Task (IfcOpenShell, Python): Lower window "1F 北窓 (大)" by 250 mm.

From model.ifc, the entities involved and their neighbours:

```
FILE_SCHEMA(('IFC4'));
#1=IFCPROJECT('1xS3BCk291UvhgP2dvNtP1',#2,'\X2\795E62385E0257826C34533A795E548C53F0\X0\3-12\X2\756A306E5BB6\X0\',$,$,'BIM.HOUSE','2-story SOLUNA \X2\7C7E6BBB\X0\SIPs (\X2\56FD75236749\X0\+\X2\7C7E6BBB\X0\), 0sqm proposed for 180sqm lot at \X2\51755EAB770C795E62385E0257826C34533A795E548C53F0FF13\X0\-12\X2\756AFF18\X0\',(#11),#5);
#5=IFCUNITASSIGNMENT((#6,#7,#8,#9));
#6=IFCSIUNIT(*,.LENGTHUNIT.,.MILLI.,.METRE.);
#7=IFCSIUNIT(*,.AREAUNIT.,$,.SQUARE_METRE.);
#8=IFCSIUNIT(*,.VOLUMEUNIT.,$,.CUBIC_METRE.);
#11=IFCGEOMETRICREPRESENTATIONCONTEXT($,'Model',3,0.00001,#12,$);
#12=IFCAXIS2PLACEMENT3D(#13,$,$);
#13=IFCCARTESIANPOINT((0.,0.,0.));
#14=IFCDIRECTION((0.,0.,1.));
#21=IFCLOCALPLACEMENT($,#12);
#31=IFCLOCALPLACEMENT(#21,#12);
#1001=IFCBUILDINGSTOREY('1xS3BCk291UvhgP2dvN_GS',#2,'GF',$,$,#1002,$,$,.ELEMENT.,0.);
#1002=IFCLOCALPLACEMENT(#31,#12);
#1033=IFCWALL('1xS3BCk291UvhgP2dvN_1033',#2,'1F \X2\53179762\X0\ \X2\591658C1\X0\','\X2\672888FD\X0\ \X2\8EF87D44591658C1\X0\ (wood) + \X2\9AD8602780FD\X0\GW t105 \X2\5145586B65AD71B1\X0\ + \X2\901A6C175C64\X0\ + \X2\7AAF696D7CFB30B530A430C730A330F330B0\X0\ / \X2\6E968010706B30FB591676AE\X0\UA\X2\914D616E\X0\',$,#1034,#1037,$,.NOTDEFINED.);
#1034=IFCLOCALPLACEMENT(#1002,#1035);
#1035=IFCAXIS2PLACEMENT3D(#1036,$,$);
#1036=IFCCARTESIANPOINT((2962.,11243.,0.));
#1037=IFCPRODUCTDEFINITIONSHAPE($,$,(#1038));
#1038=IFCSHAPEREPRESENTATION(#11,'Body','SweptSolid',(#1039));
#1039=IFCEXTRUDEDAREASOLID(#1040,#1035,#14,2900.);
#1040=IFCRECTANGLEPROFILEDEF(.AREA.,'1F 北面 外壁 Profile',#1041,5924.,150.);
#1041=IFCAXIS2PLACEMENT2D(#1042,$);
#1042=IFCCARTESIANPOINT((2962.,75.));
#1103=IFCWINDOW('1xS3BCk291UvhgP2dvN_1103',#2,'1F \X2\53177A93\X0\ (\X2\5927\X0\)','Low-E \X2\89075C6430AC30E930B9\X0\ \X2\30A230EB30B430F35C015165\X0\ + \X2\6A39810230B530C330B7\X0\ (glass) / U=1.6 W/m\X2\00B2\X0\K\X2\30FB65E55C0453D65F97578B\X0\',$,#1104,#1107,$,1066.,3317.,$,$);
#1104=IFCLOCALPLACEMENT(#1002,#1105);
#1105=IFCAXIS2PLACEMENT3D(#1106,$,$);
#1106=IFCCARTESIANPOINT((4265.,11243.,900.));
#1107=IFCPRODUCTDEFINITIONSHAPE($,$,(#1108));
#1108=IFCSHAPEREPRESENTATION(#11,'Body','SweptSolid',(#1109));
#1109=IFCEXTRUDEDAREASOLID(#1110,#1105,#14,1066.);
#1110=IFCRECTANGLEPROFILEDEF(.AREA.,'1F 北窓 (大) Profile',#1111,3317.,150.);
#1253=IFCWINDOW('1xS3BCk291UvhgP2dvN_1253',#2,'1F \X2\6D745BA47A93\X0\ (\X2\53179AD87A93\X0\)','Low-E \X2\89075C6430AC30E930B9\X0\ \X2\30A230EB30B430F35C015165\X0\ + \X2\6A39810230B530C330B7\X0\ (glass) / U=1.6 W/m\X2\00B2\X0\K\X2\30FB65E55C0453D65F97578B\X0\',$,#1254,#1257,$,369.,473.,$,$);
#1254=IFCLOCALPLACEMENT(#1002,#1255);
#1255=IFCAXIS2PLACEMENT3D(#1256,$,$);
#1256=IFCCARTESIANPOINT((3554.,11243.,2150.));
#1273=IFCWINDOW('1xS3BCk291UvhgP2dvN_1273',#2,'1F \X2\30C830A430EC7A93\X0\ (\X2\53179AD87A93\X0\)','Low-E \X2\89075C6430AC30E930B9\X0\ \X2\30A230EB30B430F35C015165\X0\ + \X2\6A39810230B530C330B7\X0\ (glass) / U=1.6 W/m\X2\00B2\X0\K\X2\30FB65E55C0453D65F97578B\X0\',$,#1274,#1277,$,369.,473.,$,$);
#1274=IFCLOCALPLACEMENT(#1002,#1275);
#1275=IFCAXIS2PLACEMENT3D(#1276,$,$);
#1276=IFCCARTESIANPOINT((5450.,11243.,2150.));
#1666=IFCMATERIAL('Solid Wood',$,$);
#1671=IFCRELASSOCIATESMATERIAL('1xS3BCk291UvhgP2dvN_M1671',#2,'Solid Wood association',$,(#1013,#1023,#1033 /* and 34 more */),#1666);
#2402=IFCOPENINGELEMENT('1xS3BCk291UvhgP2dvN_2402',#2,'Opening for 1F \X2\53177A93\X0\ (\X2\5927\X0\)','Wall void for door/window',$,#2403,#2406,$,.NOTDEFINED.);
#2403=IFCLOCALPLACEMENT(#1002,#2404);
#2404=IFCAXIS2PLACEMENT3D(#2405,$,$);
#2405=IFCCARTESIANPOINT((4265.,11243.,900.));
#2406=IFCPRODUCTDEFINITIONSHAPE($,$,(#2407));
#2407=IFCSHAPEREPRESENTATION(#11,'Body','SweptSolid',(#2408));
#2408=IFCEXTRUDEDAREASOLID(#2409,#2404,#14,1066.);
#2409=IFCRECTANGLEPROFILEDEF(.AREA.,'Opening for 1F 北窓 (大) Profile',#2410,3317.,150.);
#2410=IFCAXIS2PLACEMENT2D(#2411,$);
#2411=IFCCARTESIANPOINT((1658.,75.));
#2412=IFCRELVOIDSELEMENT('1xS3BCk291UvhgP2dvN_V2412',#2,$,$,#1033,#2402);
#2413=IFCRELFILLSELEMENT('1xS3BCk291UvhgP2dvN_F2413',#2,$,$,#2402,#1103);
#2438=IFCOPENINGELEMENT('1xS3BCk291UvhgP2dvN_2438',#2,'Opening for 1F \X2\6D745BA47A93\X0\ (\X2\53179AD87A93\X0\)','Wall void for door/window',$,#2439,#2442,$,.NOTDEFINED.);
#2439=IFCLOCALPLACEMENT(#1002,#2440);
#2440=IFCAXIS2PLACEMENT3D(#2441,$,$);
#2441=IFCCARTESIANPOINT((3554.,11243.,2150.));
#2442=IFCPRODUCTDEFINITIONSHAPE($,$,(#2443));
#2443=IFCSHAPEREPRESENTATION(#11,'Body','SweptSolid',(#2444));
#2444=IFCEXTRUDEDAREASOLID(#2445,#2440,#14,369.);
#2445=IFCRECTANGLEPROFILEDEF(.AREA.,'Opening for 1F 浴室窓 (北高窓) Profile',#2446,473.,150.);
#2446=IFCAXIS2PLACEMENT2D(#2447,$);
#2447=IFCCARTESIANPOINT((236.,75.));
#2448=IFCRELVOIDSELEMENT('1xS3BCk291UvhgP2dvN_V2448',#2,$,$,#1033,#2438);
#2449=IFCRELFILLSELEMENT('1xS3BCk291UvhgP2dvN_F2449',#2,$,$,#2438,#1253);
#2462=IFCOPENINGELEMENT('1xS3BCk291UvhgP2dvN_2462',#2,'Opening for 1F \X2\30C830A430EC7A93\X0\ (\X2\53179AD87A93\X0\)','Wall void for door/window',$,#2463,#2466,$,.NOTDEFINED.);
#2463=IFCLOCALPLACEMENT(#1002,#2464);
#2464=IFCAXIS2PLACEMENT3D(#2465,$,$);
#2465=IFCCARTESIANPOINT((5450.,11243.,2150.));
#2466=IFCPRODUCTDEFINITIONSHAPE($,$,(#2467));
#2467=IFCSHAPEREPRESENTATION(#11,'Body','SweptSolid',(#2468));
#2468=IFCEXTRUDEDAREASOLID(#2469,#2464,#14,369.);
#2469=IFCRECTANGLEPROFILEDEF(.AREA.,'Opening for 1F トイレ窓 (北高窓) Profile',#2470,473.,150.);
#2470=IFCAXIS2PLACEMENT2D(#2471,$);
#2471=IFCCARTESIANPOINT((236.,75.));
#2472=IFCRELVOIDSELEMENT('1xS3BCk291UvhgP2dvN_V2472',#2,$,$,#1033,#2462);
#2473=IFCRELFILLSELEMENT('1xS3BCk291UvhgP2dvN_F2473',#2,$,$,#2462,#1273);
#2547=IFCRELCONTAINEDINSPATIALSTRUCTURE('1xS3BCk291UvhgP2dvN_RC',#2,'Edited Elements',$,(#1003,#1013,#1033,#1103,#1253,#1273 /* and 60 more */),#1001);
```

```python
import numpy as np
import ifcopenshell
import ifcopenshell.api.geometry
import ifcopenshell.util.placement
import ifcopenshell.util.unit

model = ifcopenshell.open("model.ifc")
unit_scale = ifcopenshell.util.unit.calculate_unit_scale(model)

window = model.by_guid("1xS3BCk291UvhgP2dvN_1103")
opening = window.FillsVoids[0].RelatingOpeningElement
dz = -0.25 / unit_scale

shift = np.array([0.0, 0.0, dz])
# The window is not placed relative to its opening, so move both.
for product in (opening, window):
    matrix = ifcopenshell.util.placement.get_local_placement(product.ObjectPlacement)
    matrix[:3, 3] += shift
    ifcopenshell.api.geometry.edit_object_placement(model, product=product, matrix=matrix, is_si=False)

print(f"moved by {dz * unit_scale:+.3f} m")

model.write("model_v2.ifc")
```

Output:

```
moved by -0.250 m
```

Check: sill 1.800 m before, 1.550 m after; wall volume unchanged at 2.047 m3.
